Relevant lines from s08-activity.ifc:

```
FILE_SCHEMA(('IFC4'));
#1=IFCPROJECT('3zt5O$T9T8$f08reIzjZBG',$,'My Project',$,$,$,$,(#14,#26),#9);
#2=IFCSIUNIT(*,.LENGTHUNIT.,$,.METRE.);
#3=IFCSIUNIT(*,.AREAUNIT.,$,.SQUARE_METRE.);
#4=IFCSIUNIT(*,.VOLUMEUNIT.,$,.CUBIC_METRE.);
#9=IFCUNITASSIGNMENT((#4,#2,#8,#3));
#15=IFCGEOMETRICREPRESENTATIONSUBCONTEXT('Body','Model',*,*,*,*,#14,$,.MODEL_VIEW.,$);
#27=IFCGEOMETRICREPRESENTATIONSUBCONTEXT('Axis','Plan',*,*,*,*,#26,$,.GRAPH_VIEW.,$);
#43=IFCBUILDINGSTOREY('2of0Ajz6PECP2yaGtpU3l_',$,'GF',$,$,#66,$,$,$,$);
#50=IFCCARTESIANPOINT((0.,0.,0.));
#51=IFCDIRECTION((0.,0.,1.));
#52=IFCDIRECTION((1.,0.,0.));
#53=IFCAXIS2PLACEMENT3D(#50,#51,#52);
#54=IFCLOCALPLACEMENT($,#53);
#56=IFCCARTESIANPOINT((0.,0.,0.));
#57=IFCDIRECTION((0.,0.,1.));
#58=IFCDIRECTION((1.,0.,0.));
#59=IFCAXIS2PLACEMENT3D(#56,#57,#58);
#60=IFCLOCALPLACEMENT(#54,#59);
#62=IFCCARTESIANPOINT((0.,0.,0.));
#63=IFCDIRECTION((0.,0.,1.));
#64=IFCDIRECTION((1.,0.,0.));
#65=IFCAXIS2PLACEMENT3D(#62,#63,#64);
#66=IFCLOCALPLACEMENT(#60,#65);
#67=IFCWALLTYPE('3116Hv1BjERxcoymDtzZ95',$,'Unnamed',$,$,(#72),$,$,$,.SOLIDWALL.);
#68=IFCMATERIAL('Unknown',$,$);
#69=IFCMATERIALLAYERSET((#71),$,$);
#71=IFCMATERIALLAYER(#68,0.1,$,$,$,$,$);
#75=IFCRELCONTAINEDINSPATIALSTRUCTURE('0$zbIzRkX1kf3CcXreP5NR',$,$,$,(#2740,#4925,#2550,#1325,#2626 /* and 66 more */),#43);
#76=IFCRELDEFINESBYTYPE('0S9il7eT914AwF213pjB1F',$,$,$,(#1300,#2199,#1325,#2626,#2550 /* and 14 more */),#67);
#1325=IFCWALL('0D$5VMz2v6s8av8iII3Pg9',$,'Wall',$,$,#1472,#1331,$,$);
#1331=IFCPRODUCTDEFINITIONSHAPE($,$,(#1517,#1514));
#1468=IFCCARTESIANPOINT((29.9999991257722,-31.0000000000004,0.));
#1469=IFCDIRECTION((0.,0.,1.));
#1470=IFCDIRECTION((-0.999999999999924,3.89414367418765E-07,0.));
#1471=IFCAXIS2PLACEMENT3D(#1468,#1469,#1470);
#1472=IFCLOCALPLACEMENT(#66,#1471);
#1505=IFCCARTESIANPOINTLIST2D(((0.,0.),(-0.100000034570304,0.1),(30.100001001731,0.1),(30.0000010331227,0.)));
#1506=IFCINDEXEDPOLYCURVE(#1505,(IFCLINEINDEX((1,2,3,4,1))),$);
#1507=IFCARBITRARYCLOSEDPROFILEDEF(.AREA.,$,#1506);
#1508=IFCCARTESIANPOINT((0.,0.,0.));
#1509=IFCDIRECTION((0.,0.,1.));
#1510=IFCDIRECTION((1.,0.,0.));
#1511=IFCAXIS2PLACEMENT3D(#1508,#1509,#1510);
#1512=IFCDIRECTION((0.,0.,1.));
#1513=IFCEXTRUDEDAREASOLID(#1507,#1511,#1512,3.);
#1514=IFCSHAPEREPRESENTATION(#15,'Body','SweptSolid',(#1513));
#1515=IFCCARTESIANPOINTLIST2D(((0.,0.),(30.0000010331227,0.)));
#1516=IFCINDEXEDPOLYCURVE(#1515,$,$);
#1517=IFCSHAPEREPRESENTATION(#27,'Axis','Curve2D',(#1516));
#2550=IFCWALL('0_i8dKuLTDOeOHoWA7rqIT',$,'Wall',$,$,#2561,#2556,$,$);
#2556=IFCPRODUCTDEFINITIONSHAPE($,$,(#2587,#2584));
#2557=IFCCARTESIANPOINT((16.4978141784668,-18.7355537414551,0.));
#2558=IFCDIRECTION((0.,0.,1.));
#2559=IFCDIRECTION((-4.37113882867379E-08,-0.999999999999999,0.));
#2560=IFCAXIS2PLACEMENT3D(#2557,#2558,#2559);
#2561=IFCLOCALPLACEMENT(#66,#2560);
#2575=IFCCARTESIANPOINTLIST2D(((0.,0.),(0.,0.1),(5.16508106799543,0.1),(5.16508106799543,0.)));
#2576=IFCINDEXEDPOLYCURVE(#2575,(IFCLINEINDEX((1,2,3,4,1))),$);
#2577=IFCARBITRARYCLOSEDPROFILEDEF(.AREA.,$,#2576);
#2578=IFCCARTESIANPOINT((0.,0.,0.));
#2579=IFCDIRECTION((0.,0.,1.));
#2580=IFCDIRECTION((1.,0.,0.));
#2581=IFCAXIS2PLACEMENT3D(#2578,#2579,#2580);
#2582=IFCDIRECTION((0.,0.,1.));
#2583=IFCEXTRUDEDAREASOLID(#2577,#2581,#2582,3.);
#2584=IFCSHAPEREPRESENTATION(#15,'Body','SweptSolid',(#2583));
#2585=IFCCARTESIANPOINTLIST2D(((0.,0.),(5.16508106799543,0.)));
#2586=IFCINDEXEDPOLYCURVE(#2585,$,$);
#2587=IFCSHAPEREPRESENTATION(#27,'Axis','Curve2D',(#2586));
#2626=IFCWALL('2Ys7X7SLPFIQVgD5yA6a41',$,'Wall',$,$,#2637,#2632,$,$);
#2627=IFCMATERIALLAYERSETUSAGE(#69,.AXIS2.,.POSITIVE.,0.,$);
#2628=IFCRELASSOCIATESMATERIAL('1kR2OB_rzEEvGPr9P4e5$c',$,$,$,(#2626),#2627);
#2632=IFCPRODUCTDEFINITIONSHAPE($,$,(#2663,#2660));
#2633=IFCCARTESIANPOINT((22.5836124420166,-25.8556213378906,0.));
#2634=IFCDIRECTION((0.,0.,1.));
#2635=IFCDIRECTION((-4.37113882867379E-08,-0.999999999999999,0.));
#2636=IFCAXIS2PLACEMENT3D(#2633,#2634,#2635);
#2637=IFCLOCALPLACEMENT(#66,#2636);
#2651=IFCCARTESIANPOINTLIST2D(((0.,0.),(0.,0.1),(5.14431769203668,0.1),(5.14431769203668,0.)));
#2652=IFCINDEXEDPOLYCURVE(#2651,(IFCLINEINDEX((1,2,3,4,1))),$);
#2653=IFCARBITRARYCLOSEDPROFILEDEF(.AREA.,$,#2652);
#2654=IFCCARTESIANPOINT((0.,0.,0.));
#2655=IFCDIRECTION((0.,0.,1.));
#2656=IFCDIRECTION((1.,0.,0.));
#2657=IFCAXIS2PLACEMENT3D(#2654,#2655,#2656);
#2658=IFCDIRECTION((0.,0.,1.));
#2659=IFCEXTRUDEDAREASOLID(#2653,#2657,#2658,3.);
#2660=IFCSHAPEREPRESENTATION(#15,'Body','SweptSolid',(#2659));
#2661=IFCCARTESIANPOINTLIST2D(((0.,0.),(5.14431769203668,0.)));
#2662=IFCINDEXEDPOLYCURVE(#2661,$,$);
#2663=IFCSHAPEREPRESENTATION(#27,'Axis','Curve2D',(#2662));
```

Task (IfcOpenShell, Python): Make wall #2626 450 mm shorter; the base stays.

```python
import ifcopenshell
import ifcopenshell.geom
import ifcopenshell.util.representation
import ifcopenshell.util.shape

model = ifcopenshell.open("s08-activity.ifc")
settings = ifcopenshell.geom.settings()


def volume(element):
    """Net volume in cubic metres, openings subtracted."""
    shape = ifcopenshell.geom.create_shape(settings, element)
    return ifcopenshell.util.shape.get_volume(shape.geometry)


wall = model.by_id(2626)
before = volume(wall)

body = ifcopenshell.util.representation.get_representation(wall, "Model", "Body")
solid = body.Items[0]
old_height = solid.Depth
solid.Depth -= 0.45
after = volume(wall)

print(f"height {old_height:g} -> {solid.Depth:g}, volume {before:.3f} -> {after:.3f} m3")

model.write("s08-activity-out.ifc")
```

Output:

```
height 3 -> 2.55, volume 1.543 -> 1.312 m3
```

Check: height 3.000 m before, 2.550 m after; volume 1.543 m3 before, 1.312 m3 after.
